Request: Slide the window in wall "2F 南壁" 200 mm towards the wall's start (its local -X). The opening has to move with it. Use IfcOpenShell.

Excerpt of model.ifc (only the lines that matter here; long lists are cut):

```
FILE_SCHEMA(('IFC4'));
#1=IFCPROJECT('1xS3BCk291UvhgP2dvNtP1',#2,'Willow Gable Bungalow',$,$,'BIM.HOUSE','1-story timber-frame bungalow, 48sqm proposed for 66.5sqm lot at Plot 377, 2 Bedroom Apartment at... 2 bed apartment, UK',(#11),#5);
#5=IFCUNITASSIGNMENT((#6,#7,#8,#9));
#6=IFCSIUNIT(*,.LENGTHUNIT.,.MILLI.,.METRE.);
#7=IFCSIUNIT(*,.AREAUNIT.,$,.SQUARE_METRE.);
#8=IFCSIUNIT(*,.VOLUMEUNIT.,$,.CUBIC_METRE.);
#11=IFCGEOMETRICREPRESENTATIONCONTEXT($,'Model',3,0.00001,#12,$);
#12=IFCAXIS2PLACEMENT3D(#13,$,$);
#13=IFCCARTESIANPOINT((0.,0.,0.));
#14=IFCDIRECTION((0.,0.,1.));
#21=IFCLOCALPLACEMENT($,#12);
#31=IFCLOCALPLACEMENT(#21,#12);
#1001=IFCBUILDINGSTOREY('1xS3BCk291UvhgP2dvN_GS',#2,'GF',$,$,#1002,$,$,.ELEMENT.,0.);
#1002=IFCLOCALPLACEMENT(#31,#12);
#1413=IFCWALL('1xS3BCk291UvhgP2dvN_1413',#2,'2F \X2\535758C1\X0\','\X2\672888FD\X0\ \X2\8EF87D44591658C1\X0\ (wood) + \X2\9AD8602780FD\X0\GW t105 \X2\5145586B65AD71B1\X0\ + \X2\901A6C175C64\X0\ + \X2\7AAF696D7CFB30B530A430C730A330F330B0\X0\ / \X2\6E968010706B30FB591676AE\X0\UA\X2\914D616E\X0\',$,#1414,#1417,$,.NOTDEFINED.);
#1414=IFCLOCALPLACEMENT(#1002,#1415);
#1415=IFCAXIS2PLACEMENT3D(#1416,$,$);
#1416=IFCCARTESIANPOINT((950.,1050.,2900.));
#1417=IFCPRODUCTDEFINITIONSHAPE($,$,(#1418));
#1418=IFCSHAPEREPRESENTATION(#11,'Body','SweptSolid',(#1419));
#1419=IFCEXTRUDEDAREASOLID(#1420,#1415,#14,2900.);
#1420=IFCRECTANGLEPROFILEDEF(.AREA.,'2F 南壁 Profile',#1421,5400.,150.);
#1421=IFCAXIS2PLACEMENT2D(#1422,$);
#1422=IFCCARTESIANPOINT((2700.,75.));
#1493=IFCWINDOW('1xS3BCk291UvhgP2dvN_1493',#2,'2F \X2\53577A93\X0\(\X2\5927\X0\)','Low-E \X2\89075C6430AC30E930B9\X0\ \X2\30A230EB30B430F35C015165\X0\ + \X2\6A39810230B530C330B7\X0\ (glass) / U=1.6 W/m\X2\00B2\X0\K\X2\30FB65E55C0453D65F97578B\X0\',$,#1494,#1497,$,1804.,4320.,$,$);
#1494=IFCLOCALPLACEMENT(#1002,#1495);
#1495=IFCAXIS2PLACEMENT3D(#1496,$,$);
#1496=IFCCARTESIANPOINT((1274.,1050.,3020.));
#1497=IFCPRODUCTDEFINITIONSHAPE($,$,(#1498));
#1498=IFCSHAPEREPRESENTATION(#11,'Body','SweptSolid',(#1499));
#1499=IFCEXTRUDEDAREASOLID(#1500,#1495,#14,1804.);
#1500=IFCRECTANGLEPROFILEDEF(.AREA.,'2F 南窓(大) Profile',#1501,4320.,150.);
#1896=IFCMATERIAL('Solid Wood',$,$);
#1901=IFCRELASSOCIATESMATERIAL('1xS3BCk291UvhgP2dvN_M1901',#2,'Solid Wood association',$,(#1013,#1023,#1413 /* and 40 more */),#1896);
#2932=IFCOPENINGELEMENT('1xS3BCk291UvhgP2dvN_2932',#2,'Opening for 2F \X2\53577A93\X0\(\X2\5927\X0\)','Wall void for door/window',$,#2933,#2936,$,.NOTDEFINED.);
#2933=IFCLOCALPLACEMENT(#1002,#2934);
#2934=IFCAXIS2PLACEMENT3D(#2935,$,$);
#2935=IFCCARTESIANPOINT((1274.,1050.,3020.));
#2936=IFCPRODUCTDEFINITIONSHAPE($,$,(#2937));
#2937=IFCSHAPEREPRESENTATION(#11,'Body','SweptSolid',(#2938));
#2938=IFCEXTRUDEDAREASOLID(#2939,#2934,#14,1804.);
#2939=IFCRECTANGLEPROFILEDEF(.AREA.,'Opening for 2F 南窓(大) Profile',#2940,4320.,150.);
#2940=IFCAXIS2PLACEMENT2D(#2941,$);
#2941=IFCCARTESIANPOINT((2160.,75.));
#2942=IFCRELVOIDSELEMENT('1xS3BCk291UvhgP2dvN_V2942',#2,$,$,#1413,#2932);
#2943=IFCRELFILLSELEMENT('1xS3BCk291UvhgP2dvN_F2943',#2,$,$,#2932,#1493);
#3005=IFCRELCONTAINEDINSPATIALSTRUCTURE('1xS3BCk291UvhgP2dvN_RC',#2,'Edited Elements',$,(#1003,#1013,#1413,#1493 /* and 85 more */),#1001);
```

```python
import ifcopenshell
import ifcopenshell.api.geometry
import ifcopenshell.util.placement
import ifcopenshell.util.unit

model = ifcopenshell.open("model.ifc")
unit_scale = ifcopenshell.util.unit.calculate_unit_scale(model)

window = model.by_guid("1xS3BCk291UvhgP2dvN_1493")
opening = window.FillsVoids[0].RelatingOpeningElement
wall = opening.VoidsElements[0].RelatingBuildingElement

wall_matrix = ifcopenshell.util.placement.get_local_placement(wall.ObjectPlacement)
shift = wall_matrix[:3, 0] * -0.2 / unit_scale
before = ifcopenshell.util.placement.get_local_placement(window.ObjectPlacement)[:3, 3].copy()

# The window is not placed relative to its opening, so move both.
for product in (opening, window):
    matrix = ifcopenshell.util.placement.get_local_placement(product.ObjectPlacement)
    matrix[:3, 3] += shift
    ifcopenshell.api.geometry.edit_object_placement(model, product=product, matrix=matrix, is_si=False)

after = ifcopenshell.util.placement.get_local_placement(window.ObjectPlacement)[:3, 3]
print("window moved by", (after - before).round(3) + 0.0)

model.write("model-out.ifc")
```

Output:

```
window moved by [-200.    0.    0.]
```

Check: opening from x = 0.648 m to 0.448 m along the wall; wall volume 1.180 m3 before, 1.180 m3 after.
